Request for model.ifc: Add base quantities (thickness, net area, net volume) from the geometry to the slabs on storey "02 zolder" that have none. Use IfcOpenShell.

First a look at what the model holds.

```python
import ifcopenshell
import ifcopenshell.util.element
import ifcopenshell.util.unit

model = ifcopenshell.open("model.ifc")
print(model.schema)
for unit_type in ("LENGTHUNIT", "AREAUNIT", "VOLUMEUNIT"):
    print(unit_type, ifcopenshell.util.unit.calculate_unit_scale(model, unit_type))
storey = next(s for s in model.by_type("IfcBuildingStorey") if s.Name == "02 zolder")
slabs = [e for e in ifcopenshell.util.element.get_decomposition(storey) if e.is_a("IfcSlab")]
for e in sorted(slabs, key=lambda e: e.id()):
    print(e.id(), e.is_a(), e.Name, list(ifcopenshell.util.element.get_psets(e, qtos_only=True)), sep=" | ")
```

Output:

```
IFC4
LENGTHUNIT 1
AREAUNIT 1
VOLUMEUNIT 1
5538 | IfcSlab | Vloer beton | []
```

```python
import ifcopenshell
import ifcopenshell.api.pset
import ifcopenshell.geom
import ifcopenshell.util.element
import ifcopenshell.util.shape
import ifcopenshell.util.unit

model = ifcopenshell.open("model.ifc")
unit_scale = ifcopenshell.util.unit.calculate_unit_scale(model)
area_scale = ifcopenshell.util.unit.calculate_unit_scale(model, "AREAUNIT")
volume_scale = ifcopenshell.util.unit.calculate_unit_scale(model, "VOLUMEUNIT")
settings = ifcopenshell.geom.settings()

storey = next(s for s in model.by_type("IfcBuildingStorey") if s.Name == "02 zolder")
slabs = [e for e in ifcopenshell.util.element.get_decomposition(storey) if e.is_a("IfcSlab")]

for e in sorted(slabs, key=lambda e: e.id()):
    if ifcopenshell.util.element.get_psets(e, qtos_only=True, should_inherit=False):
        continue
    # Geometry comes back in metres, in the element's own axes.
    shape = ifcopenshell.geom.create_shape(settings, e)
    values = {
        "Width": ifcopenshell.util.shape.get_z(shape.geometry) / unit_scale,
        "NetArea": ifcopenshell.util.shape.get_footprint_area(shape.geometry) / area_scale,
        "NetVolume": ifcopenshell.util.shape.get_volume(shape.geometry) / volume_scale,
    }
    qto = ifcopenshell.api.pset.add_qto(model, product=e, name="Qto_SlabBaseQuantities")
    ifcopenshell.api.pset.edit_qto(model, qto=qto, properties=values)
    print(e.id(), {k: round(v, 3) for k, v in values.items()})

model.write("model_rev.ifc")
```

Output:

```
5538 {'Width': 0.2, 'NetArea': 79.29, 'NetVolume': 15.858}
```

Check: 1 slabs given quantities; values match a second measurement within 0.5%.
